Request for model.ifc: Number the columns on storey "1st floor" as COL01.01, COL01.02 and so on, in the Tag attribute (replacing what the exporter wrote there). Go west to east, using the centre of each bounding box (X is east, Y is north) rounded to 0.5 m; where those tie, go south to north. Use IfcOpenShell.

First a look at what the model holds.

```python
import ifcopenshell
import ifcopenshell.util.element
import ifcopenshell.util.placement

model = ifcopenshell.open("model.ifc")
print(model.schema)
storey = next(s for s in model.by_type("IfcBuildingStorey") if s.Name == "1st floor")
columns = [e for e in ifcopenshell.util.element.get_decomposition(storey) if e.is_a("IfcColumn")]
for e in sorted(columns, key=lambda e: e.id()):
    origin = ifcopenshell.util.placement.get_local_placement(e.ObjectPlacement)[:3, 3]
    print(e.id(), e.Tag, e.Name, origin.round(2) + 0.0, sep=" | ")
```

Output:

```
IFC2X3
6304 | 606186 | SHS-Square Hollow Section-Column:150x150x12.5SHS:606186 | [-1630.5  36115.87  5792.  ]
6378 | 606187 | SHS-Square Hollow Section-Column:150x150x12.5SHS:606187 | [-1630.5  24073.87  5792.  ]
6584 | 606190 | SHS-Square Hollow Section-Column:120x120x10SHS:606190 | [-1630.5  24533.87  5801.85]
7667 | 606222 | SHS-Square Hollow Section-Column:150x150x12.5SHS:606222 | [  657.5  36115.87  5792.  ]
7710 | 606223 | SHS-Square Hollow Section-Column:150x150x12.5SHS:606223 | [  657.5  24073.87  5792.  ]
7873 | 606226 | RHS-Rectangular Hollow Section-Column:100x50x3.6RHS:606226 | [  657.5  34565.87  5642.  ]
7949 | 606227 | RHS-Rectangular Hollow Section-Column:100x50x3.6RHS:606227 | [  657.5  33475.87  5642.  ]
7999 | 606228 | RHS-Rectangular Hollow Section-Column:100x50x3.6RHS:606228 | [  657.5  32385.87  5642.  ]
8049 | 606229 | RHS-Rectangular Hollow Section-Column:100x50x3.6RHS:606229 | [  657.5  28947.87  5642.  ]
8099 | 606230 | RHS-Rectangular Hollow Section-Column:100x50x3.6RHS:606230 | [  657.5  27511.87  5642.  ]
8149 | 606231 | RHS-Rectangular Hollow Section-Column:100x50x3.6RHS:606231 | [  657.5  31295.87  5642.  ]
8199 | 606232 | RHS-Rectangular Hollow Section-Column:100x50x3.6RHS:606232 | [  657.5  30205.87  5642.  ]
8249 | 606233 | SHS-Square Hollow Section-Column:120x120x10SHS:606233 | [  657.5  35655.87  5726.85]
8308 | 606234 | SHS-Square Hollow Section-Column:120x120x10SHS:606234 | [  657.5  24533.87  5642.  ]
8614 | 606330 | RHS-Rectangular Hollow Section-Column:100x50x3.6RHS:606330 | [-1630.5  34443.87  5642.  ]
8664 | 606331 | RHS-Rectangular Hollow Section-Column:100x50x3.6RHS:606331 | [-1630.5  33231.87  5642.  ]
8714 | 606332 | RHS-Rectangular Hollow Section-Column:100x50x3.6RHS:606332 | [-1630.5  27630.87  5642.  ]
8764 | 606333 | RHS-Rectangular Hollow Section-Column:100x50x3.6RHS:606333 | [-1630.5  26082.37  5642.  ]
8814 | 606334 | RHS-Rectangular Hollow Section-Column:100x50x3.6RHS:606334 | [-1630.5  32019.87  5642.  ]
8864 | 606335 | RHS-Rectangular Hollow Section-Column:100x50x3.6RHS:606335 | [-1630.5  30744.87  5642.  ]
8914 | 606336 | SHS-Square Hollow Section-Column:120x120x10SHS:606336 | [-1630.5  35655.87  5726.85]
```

```python
import ifcopenshell
import ifcopenshell.geom
import ifcopenshell.util.element
import ifcopenshell.util.shape

model = ifcopenshell.open("model.ifc")
settings = ifcopenshell.geom.settings()
settings.set("use-world-coords", True)


def centre(element):
    shape = ifcopenshell.geom.create_shape(settings, element)
    return ifcopenshell.util.shape.get_bbox_centroid(shape.geometry)


storey = next(s for s in model.by_type("IfcBuildingStorey") if s.Name == "1st floor")
columns = [e for e in ifcopenshell.util.element.get_decomposition(storey) if e.is_a("IfcColumn")]

# Insertion points can sit at a corner or the storey origin, so sort by the geometry (in metres).
centres = {e: centre(e) for e in columns}
columns.sort(key=lambda e: (round(centres[e][0] / 0.5), centres[e][1]))

for i, e in enumerate(columns, start=1):
    number = f"COL01.{i:02d}"
    e.Tag = number
    print(e.id(), number)

model.write("model_edited.ifc")
```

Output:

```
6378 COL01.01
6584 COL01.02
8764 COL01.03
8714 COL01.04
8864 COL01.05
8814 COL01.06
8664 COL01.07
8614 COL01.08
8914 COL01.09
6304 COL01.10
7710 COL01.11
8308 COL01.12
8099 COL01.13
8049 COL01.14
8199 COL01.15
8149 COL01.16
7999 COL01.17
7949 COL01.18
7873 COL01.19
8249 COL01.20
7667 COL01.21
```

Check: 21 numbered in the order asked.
